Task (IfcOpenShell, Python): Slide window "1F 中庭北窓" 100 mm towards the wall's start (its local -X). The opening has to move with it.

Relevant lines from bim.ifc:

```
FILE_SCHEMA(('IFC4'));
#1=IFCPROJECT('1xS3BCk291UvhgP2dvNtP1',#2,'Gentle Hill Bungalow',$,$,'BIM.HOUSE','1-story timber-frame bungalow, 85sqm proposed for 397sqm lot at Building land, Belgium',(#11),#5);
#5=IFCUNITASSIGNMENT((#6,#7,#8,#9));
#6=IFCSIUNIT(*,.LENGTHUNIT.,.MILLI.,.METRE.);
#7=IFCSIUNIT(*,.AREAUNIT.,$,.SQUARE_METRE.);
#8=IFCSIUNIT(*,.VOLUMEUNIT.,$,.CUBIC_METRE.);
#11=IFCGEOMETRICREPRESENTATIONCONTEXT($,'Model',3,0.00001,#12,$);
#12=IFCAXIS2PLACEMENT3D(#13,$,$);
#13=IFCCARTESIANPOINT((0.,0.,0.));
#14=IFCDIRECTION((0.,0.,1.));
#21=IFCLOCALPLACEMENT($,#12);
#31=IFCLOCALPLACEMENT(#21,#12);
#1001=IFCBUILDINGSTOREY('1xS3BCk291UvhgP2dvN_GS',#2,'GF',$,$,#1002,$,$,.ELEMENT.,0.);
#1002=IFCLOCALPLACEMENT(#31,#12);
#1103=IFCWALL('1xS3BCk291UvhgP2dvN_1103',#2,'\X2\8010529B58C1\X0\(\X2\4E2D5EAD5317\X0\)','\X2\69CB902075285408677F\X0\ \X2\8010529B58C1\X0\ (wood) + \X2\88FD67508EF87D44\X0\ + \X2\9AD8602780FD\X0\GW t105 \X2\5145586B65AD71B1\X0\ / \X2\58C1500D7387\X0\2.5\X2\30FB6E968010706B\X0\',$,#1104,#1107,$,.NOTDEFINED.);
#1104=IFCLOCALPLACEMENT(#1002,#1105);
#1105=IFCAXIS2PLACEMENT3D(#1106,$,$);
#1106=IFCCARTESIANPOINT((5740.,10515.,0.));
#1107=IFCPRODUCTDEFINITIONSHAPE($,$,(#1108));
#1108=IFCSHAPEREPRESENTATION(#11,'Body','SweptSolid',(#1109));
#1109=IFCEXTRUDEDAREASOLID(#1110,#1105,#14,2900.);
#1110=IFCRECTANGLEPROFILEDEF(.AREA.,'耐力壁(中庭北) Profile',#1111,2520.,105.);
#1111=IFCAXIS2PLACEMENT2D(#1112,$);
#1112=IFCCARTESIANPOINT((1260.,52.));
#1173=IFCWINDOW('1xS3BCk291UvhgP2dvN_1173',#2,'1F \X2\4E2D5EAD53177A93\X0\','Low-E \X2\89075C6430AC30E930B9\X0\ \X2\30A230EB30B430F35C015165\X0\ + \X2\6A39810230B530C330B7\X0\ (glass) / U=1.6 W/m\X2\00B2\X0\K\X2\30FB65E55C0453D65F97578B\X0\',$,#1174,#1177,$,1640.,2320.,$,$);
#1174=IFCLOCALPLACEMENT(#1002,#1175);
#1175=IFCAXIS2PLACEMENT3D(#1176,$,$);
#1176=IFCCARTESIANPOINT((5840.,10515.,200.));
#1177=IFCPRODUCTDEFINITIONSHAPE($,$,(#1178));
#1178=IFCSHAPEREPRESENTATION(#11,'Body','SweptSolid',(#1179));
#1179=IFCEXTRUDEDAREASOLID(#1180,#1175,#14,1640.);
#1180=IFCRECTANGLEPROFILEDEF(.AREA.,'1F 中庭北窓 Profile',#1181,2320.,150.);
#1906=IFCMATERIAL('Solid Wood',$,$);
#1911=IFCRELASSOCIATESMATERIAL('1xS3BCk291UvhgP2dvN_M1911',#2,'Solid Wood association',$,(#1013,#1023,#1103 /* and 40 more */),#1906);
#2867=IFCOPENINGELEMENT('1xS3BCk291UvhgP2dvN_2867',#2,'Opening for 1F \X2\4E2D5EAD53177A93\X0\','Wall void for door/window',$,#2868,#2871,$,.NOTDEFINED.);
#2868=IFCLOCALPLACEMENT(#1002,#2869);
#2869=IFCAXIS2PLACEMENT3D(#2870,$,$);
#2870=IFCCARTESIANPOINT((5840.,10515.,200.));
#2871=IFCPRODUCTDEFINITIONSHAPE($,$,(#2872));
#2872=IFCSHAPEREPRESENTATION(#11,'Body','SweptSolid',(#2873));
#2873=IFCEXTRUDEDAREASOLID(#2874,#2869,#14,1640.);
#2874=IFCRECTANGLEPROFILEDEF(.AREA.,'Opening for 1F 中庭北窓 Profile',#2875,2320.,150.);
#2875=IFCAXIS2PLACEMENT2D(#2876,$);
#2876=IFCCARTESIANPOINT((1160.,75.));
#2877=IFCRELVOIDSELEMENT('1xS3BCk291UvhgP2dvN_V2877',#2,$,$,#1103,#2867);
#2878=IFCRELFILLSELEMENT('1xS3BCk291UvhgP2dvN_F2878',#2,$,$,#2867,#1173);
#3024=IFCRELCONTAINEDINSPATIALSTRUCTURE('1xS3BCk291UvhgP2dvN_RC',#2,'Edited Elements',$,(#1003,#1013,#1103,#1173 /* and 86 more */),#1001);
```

```python
import ifcopenshell
import ifcopenshell.api.geometry
import ifcopenshell.util.placement

model = ifcopenshell.open("bim.ifc")

window = model.by_id(1173)
opening = window.FillsVoids[0].RelatingOpeningElement
wall = opening.VoidsElements[0].RelatingBuildingElement

wall_matrix = ifcopenshell.util.placement.get_local_placement(wall.ObjectPlacement)
shift = wall_matrix[:3, 0] * -100.0
before = ifcopenshell.util.placement.get_local_placement(window.ObjectPlacement)[:3, 3].copy()

# The window is not placed relative to its opening, so move both.
for product in (opening, window):
    matrix = ifcopenshell.util.placement.get_local_placement(product.ObjectPlacement)
    matrix[:3, 3] += shift
    ifcopenshell.api.geometry.edit_object_placement(model, product=product, matrix=matrix, is_si=False)

after = ifcopenshell.util.placement.get_local_placement(window.ObjectPlacement)[:3, 3]
print("window moved by", (after - before).round(3) + 0.0)

model.write("bim_edited.ifc")
```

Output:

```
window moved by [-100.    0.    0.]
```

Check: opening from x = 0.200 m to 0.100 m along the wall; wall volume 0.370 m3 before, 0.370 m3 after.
